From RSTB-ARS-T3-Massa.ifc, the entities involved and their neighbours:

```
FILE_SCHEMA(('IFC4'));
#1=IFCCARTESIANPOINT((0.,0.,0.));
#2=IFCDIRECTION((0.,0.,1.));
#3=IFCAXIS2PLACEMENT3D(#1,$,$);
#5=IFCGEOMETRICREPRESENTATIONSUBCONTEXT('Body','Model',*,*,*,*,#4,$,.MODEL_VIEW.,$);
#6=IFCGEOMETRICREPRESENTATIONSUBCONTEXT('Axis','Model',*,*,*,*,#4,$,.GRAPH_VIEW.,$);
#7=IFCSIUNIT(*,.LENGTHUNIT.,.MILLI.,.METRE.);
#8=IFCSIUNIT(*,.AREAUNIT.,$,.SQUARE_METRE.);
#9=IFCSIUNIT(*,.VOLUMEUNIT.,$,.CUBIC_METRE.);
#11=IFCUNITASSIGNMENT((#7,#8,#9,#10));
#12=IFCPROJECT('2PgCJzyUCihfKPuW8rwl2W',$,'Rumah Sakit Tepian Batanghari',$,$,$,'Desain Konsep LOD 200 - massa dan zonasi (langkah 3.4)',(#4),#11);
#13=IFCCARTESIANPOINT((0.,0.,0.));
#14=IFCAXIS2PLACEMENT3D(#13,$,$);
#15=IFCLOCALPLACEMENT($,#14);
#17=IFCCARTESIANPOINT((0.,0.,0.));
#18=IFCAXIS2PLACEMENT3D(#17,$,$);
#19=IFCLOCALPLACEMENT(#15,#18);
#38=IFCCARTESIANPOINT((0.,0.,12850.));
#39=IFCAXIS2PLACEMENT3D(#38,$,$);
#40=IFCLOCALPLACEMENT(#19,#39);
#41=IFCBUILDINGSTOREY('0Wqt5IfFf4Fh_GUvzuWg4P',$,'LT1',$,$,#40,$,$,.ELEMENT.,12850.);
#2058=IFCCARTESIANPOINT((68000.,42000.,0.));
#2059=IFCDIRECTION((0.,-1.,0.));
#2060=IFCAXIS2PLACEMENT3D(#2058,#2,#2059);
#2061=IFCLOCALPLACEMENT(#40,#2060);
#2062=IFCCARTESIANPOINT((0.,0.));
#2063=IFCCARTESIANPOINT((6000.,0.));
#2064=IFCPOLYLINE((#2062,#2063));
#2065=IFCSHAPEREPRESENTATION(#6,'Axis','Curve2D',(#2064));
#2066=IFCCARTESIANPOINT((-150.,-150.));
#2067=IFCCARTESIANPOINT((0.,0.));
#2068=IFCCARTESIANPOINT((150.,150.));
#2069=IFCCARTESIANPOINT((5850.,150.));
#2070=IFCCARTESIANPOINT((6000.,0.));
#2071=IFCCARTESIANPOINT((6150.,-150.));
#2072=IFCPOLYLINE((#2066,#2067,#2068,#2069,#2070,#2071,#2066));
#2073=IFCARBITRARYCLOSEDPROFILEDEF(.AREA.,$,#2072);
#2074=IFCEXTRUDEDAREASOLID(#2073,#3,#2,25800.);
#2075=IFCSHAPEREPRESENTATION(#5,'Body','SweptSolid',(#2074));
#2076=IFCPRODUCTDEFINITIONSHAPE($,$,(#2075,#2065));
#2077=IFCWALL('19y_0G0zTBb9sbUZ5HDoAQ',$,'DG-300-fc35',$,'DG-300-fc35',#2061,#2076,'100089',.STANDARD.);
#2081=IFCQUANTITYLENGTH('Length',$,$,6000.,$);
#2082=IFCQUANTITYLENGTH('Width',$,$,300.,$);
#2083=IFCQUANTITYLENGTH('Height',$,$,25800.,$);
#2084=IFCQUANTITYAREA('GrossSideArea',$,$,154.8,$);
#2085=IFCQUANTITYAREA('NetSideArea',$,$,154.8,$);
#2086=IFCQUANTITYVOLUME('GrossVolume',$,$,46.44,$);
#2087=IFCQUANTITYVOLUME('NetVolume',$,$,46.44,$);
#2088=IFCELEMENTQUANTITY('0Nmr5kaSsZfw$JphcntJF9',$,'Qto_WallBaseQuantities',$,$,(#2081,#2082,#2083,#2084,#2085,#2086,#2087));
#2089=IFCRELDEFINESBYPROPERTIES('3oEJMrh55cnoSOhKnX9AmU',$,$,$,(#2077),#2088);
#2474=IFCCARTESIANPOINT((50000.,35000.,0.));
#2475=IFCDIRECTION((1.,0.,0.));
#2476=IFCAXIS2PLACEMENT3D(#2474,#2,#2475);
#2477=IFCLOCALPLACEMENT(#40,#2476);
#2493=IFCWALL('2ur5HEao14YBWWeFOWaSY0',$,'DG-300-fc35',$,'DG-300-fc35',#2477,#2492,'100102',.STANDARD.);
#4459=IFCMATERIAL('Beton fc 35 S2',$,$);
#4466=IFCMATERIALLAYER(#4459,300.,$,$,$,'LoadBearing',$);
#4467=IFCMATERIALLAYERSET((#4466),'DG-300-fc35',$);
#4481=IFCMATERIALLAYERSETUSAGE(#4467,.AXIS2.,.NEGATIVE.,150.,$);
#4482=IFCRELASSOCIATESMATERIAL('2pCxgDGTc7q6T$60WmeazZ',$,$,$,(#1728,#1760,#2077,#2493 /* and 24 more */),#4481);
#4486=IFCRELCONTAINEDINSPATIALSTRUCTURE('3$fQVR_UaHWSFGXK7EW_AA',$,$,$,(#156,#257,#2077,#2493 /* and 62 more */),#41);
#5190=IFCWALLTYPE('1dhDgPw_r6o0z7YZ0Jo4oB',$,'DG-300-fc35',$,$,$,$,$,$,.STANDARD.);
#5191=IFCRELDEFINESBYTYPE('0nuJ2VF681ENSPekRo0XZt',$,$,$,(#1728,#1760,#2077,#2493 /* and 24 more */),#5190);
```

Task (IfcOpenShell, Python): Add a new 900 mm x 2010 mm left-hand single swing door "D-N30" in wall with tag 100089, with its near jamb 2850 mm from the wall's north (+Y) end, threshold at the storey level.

```python
import numpy as np
import ifcopenshell
import ifcopenshell.api.feature
import ifcopenshell.api.geometry
import ifcopenshell.api.pset
import ifcopenshell.api.root
import ifcopenshell.api.spatial
import ifcopenshell.geom
import ifcopenshell.util.element
import ifcopenshell.util.placement
import ifcopenshell.util.representation
import ifcopenshell.util.shape
import ifcopenshell.util.unit

model = ifcopenshell.open("RSTB-ARS-T3-Massa.ifc")
unit_scale = ifcopenshell.util.unit.calculate_unit_scale(model)
area_scale = ifcopenshell.util.unit.calculate_unit_scale(model, "AREAUNIT")
volume_scale = ifcopenshell.util.unit.calculate_unit_scale(model, "VOLUMEUNIT")
settings = ifcopenshell.geom.settings()


def volume(element):
    """Net volume in cubic metres, openings subtracted."""
    shape = ifcopenshell.geom.create_shape(settings, element)
    return ifcopenshell.util.shape.get_volume(shape.geometry)


wall = model.by_guid("19y_0G0zTBb9sbUZ5HDoAQ")
storey = ifcopenshell.util.element.get_container(wall, ifc_class="IfcBuildingStorey")
context = ifcopenshell.util.representation.get_context(model, "Model", "Body", "MODEL_VIEW")
before = volume(wall)

width, height, from_end, sill = 0.9, 2.01, 2.85, 0.0  # metres

# The wall runs along its own X axis, and the end named is its -X end.
wall_shape = ifcopenshell.geom.create_shape(settings, wall)
x, y, z = ifcopenshell.util.shape.get_vertices(wall_shape.geometry).T
start = x.min() + from_end
face, thickness = float(y.min()), float(y.max() - y.min())
wall_matrix = ifcopenshell.util.placement.get_local_placement(wall.ObjectPlacement)
level = ifcopenshell.util.placement.get_local_placement(storey.ObjectPlacement)[2, 3]


def in_wall(x, y):
    """Placement at x, y metres in the wall's axes, at sill height."""
    matrix = wall_matrix.copy()
    matrix[:, 3] = wall_matrix @ np.array([x / unit_scale, y / unit_scale, 0.0, 1.0])
    matrix[2, 3] = level + sill / unit_scale
    return matrix


# Opening: a box that overshoots both wall faces by 50 mm.
opening = ifcopenshell.api.root.create_entity(model, ifc_class="IfcOpeningElement", predefined_type="OPENING")
box = ifcopenshell.api.geometry.add_wall_representation(
    model, context=context, length=width, height=height, thickness=thickness + 0.1
)
ifcopenshell.api.geometry.assign_representation(model, product=opening, representation=box)
ifcopenshell.api.geometry.edit_object_placement(model, product=opening, matrix=in_wall(start, face - 0.05), is_si=False)
ifcopenshell.api.feature.add_feature(model, feature=opening, element=wall)

door = ifcopenshell.api.root.create_entity(model, ifc_class="IfcDoor", name="D-N30", predefined_type="DOOR")
door.OverallWidth, door.OverallHeight = width / unit_scale, height / unit_scale
door.OperationType = "SINGLE_SWING_LEFT"
body = ifcopenshell.api.geometry.add_door_representation(
    model,
    context=context,
    overall_width=door.OverallWidth,
    overall_height=door.OverallHeight,
    operation_type="SINGLE_SWING_LEFT",
    lining_properties={"LiningDepth": thickness / unit_scale, "ThresholdDepth": thickness / unit_scale},
)
ifcopenshell.api.geometry.assign_representation(model, product=door, representation=body)
ifcopenshell.api.spatial.assign_container(model, products=[door], relating_structure=storey)
ifcopenshell.api.feature.add_filling(model, opening=opening, element=door)

# The lining spans the wall, so the door starts at the wall face.
ifcopenshell.api.geometry.edit_object_placement(model, product=door, matrix=in_wall(start, face), is_si=False)

after = volume(wall)

# Update the wall's stored quantities.
qto = model.by_id(ifcopenshell.util.element.get_pset(wall, "Qto_WallBaseQuantities", should_inherit=False)["id"])
ifcopenshell.api.pset.edit_qto(model, qto=qto, properties={
    "NetSideArea": after / thickness / area_scale,
    "NetVolume": after / volume_scale,
})

print(f"wall volume {before:.3f} -> {after:.3f} m3")

model.write("RSTB-ARS-T3-Massa_updated.ifc")
```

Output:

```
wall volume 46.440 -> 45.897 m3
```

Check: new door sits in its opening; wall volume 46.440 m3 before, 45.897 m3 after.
